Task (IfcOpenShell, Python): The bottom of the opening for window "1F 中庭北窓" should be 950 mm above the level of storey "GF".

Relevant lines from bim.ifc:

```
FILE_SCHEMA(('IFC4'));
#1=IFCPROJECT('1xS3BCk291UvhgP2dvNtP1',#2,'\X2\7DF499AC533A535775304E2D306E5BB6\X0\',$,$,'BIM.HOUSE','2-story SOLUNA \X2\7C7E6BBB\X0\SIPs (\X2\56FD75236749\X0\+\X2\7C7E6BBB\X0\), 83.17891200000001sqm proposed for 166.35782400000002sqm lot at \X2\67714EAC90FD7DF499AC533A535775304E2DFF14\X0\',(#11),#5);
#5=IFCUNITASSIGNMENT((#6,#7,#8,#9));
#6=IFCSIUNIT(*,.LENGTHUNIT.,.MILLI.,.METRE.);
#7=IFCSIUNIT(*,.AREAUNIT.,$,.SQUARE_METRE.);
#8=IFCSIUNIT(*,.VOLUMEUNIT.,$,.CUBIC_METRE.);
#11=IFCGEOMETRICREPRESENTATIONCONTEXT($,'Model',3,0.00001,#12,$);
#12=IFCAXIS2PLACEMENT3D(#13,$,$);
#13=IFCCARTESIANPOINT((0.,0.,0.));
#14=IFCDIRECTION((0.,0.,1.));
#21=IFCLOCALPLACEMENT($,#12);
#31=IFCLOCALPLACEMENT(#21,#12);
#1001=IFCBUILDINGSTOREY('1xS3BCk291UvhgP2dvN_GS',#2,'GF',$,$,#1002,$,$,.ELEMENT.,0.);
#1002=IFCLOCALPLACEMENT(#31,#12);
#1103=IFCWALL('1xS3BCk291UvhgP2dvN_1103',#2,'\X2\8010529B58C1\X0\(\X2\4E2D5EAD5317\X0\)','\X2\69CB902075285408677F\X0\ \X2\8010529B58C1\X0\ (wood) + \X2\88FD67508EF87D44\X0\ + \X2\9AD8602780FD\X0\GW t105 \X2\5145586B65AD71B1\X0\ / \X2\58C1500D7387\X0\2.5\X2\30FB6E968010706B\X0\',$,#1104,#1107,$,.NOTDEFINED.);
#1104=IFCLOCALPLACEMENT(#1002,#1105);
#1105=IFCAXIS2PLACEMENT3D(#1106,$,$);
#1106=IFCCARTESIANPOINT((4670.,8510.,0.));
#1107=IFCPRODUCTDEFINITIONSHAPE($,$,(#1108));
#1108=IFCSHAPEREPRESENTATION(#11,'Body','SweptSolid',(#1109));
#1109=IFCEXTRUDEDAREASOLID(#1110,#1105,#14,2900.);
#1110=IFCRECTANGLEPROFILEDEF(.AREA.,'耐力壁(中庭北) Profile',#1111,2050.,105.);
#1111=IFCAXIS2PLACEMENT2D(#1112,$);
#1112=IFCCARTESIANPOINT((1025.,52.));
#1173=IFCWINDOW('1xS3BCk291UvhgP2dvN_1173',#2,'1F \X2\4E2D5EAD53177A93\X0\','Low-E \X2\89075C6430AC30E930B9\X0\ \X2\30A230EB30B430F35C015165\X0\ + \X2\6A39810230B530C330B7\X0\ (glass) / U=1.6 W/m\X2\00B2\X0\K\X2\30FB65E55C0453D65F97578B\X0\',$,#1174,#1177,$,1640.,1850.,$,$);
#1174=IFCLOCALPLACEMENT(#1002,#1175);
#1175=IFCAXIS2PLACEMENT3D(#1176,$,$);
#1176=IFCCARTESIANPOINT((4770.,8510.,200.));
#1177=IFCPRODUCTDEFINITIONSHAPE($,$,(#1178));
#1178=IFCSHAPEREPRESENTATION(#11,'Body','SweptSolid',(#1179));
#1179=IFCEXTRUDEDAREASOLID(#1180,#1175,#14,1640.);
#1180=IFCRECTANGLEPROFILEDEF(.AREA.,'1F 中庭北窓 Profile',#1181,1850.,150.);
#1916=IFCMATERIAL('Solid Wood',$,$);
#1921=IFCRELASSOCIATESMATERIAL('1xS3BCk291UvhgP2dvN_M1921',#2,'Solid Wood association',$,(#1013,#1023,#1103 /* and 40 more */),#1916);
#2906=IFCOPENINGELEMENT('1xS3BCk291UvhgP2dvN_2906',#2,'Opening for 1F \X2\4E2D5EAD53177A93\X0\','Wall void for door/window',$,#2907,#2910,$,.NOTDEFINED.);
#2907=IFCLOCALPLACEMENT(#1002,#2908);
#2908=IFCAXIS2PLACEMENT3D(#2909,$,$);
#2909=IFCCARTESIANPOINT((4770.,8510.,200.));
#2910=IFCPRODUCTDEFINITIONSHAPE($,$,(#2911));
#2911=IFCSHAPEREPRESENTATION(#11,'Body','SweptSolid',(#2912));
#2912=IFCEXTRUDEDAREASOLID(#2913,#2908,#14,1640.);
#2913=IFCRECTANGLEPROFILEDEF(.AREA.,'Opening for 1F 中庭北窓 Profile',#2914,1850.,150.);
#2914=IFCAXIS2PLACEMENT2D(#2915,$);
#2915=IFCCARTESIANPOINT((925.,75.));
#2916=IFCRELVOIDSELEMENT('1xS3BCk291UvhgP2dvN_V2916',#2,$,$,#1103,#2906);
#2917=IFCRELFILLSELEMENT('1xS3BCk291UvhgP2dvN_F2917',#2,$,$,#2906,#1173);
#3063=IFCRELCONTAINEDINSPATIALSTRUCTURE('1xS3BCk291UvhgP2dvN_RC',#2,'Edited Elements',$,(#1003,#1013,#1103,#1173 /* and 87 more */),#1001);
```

```python
import numpy as np
import ifcopenshell
import ifcopenshell.api.geometry
import ifcopenshell.geom
import ifcopenshell.util.element
import ifcopenshell.util.placement
import ifcopenshell.util.shape
import ifcopenshell.util.unit

model = ifcopenshell.open("bim.ifc")
unit_scale = ifcopenshell.util.unit.calculate_unit_scale(model)

window = model.by_guid("1xS3BCk291UvhgP2dvN_1173")
opening = window.FillsVoids[0].RelatingOpeningElement
storey = ifcopenshell.util.element.get_container(window, ifc_class="IfcBuildingStorey")
level = ifcopenshell.util.placement.get_local_placement(storey.ObjectPlacement)[2, 3]

# The opening's origin need not be at the sill, so measure its lowest point.
shape = ifcopenshell.geom.create_shape(ifcopenshell.geom.settings(), opening)
bottom = ifcopenshell.util.shape.get_shape_bottom_elevation(shape, shape.geometry) / unit_scale
dz = level + 0.95 / unit_scale - bottom

shift = np.array([0.0, 0.0, dz])
# The window is not placed relative to its opening, so move both.
for product in (opening, window):
    matrix = ifcopenshell.util.placement.get_local_placement(product.ObjectPlacement)
    matrix[:3, 3] += shift
    ifcopenshell.api.geometry.edit_object_placement(model, product=product, matrix=matrix, is_si=False)

print(f"moved by {dz * unit_scale:+.3f} m")

model.write("bim_edited.ifc")
```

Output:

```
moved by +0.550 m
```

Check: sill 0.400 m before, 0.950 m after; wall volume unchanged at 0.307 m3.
